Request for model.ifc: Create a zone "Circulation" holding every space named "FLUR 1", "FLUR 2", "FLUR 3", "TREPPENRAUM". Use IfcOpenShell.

First a look at what the model holds.

```python
import ifcopenshell

model = ifcopenshell.open("model.ifc")
print(model.schema)
seen = {}
for space in model.by_type("IfcSpace"):
    seen[space.LongName] = seen.get(space.LongName, 0) + 1
for name, count in sorted(seen.items(), key=str):
    print(count, "x", name)
print("zones:", [z.Name for z in model.by_type("IfcZone")][:20])
```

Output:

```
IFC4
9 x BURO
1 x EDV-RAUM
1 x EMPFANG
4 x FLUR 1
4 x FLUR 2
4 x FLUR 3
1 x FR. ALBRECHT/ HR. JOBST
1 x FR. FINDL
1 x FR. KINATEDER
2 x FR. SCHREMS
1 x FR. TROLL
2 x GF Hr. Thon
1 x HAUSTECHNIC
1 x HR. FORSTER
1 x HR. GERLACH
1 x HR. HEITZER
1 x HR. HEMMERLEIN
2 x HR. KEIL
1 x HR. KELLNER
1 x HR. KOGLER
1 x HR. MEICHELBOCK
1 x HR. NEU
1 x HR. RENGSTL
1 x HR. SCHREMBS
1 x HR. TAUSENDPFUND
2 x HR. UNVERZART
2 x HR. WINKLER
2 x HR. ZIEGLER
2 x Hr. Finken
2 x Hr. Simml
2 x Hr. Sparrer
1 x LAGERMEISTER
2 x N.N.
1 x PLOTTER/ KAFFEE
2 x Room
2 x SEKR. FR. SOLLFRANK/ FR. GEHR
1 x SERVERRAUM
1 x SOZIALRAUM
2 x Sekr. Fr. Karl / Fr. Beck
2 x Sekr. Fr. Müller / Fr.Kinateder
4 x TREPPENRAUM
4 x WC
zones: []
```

```python
import ifcopenshell
import ifcopenshell.api.group
import ifcopenshell.api.root

model = ifcopenshell.open("model.ifc")

names = {"FLUR 1", "FLUR 2", "FLUR 3", "TREPPENRAUM"}
spaces = [s for s in model.by_type("IfcSpace") if s.LongName in names]

zone = ifcopenshell.api.root.create_entity(model, ifc_class="IfcZone", name="Circulation")
ifcopenshell.api.group.assign_group(model, products=spaces, group=zone)
print(len(spaces), "spaces in", zone.Name)

model.write("model_edited.ifc")
```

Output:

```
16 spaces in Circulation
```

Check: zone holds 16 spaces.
